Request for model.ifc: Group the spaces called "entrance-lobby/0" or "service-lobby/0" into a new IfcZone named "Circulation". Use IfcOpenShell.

First a look at what the model holds.

```python
import ifcopenshell

model = ifcopenshell.open("model.ifc")
print(model.schema)
seen = {}
for space in model.by_type("IfcSpace"):
    seen[space.Name] = seen.get(space.Name, 0) + 1
for name, count in sorted(seen.items(), key=str):
    print(count, "x", name)
print("zones:", [z.Name for z in model.by_type("IfcZone")][:20])
```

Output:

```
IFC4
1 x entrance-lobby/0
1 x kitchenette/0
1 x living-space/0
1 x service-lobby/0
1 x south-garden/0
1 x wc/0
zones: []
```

```python
import ifcopenshell
import ifcopenshell.api.group
import ifcopenshell.api.root

model = ifcopenshell.open("model.ifc")

names = {"entrance-lobby/0", "service-lobby/0"}
spaces = [s for s in model.by_type("IfcSpace") if s.Name in names]

zone = ifcopenshell.api.root.create_entity(model, ifc_class="IfcZone", name="Circulation")
ifcopenshell.api.group.assign_group(model, products=spaces, group=zone)
print(len(spaces), "spaces in", zone.Name)

model.write("model_edited.ifc")
```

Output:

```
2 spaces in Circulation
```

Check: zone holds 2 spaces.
